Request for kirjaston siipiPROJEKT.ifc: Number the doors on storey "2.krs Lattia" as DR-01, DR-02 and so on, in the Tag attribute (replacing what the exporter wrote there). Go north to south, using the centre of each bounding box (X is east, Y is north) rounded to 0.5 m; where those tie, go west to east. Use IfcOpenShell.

First a look at what the model holds.

```python
import ifcopenshell
import ifcopenshell.util.element
import ifcopenshell.util.placement

model = ifcopenshell.open("kirjaston siipiPROJEKT.ifc")
print(model.schema)
storey = next(s for s in model.by_type("IfcBuildingStorey") if s.Name == "2.krs Lattia")
doors = [e for e in ifcopenshell.util.element.get_decomposition(storey) if e.is_a("IfcDoor")]
for e in sorted(doors, key=lambda e: e.id()):
    origin = ifcopenshell.util.placement.get_local_placement(e.ObjectPlacement)[:3, 3]
    print(e.id(), e.Tag, e.Name, origin.round(2) + 0.0, sep=" | ")
```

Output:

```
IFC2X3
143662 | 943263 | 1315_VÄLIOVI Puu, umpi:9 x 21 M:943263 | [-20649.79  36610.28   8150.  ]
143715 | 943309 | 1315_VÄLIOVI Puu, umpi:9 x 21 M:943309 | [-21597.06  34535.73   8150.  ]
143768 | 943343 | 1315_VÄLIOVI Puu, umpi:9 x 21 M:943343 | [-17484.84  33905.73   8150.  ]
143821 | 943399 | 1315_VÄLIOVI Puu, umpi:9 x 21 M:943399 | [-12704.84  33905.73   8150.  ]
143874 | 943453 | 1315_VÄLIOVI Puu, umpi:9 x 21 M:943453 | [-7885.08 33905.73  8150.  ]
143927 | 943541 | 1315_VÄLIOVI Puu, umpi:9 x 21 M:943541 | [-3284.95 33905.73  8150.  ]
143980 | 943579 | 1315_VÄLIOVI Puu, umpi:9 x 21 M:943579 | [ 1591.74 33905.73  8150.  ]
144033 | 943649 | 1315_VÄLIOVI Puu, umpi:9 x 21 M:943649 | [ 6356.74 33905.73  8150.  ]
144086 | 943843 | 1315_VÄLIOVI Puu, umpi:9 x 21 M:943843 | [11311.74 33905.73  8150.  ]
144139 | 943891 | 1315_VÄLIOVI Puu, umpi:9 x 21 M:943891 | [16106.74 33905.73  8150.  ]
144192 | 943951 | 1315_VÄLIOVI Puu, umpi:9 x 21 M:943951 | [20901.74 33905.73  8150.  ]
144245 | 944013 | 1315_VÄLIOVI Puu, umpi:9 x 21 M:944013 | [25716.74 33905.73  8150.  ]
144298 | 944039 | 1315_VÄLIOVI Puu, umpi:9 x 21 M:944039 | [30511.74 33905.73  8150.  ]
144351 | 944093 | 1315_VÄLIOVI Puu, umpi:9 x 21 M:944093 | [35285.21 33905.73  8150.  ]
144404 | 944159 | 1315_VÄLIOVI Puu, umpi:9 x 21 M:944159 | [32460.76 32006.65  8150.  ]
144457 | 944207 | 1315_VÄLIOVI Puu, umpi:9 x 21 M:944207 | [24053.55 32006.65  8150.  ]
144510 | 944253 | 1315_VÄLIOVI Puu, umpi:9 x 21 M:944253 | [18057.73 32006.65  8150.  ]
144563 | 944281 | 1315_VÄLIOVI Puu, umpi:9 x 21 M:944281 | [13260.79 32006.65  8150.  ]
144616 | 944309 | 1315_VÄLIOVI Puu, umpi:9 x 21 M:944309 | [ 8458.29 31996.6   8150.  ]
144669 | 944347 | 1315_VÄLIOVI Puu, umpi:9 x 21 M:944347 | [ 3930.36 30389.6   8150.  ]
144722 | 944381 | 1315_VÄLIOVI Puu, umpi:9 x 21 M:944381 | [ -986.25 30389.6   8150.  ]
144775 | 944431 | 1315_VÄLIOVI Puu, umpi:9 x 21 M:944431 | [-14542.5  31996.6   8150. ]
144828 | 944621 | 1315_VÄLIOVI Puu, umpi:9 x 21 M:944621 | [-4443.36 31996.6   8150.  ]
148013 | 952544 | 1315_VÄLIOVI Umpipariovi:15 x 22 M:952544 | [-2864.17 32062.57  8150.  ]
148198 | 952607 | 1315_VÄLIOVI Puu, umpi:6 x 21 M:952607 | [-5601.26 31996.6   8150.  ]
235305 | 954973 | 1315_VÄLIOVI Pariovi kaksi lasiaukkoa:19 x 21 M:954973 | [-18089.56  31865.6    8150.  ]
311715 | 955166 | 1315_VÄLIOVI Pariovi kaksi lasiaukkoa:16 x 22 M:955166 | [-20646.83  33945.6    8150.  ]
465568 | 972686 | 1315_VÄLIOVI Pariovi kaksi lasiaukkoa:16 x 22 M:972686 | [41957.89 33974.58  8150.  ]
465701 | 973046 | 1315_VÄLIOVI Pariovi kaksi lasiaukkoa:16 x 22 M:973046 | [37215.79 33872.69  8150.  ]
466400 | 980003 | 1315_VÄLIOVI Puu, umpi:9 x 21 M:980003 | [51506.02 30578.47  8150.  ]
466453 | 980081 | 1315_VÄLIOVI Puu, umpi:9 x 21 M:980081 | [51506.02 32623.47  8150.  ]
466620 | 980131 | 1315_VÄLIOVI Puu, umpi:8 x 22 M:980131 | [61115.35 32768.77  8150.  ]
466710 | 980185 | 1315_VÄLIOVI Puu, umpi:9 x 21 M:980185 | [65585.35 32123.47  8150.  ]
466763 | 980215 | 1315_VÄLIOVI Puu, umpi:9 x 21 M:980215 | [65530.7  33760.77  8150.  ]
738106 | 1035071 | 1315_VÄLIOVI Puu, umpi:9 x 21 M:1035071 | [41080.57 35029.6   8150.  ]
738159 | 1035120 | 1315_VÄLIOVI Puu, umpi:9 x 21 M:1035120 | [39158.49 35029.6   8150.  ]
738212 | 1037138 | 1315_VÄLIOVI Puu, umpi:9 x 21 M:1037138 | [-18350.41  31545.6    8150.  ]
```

```python
import ifcopenshell
import ifcopenshell.geom
import ifcopenshell.util.element
import ifcopenshell.util.shape

model = ifcopenshell.open("kirjaston siipiPROJEKT.ifc")
settings = ifcopenshell.geom.settings()
settings.set("use-world-coords", True)


def centre(element):
    shape = ifcopenshell.geom.create_shape(settings, element)
    return ifcopenshell.util.shape.get_bbox_centroid(shape.geometry)


storey = next(s for s in model.by_type("IfcBuildingStorey") if s.Name == "2.krs Lattia")
doors = [e for e in ifcopenshell.util.element.get_decomposition(storey) if e.is_a("IfcDoor")]

# Insertion points can sit at a corner or the storey origin, so sort by the geometry (in metres).
centres = {e: centre(e) for e in doors}
doors.sort(key=lambda e: (-round(centres[e][1] / 0.5), centres[e][0]))

for i, e in enumerate(doors, start=1):
    number = f"DR-{i:02d}"
    e.Tag = number
    print(e.id(), number)

model.write("kirjaston siipiPROJEKT_rev.ifc")
```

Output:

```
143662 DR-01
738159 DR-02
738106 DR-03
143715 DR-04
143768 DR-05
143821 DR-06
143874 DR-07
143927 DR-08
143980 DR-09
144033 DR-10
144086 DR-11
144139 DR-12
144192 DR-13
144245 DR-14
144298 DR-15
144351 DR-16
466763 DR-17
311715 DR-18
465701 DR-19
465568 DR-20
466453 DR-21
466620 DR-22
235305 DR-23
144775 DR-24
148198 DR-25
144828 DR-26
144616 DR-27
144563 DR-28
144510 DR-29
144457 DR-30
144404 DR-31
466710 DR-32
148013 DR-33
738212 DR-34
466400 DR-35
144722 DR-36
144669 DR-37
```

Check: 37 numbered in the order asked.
